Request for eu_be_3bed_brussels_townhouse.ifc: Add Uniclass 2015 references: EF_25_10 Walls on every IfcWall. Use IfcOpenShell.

First a look at what the model holds.

```python
import ifcopenshell

model = ifcopenshell.open("eu_be_3bed_brussels_townhouse.ifc")
print(model.schema)
print("classifications:", [c.Name for c in model.by_type("IfcClassification")])
for ifc_class in ("IfcDoor", "IfcRoof", "IfcStair", "IfcWall", "IfcWindow"):
    print(ifc_class, len(model.by_type(ifc_class)))
```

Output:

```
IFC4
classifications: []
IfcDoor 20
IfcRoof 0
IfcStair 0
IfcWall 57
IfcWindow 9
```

```python
import ifcopenshell
import ifcopenshell.api.classification

model = ifcopenshell.open("eu_be_3bed_brussels_townhouse.ifc")

system = ifcopenshell.api.classification.add_classification(model, classification="Uniclass 2015")

codes = {
    "IfcWall": ("EF_25_10", "Walls"),
}
for ifc_class, (code, name) in codes.items():
    products = model.by_type(ifc_class)
    ifcopenshell.api.classification.add_reference(
        model, products=products, classification=system, identification=code, name=name
    )
    print(code, len(products))

model.write("eu_be_3bed_brussels_townhouse-out.ifc")
```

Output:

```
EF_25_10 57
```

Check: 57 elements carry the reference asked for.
